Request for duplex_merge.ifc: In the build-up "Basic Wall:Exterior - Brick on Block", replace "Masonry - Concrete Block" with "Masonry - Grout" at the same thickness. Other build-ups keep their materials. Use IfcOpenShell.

First a look at what the model holds.

```python
import ifcopenshell
import ifcopenshell.util.element

model = ifcopenshell.open("duplex_merge.ifc")
print(model.schema)
for layer_set in model.by_type("IfcMaterialLayerSet"):
    if layer_set.LayerSetName == "Basic Wall:Exterior - Brick on Block":
        for layer in layer_set.MaterialLayers:
            print(layer.id(), layer.Material and layer.Material.Name, layer.LayerThickness, sep=" | ")
        print(len(ifcopenshell.util.element.get_elements_by_material(model, layer_set)), "elements and types use it")
print(sorted(m.Name for m in model.by_type("IfcMaterial") if m.Name)[:60])
```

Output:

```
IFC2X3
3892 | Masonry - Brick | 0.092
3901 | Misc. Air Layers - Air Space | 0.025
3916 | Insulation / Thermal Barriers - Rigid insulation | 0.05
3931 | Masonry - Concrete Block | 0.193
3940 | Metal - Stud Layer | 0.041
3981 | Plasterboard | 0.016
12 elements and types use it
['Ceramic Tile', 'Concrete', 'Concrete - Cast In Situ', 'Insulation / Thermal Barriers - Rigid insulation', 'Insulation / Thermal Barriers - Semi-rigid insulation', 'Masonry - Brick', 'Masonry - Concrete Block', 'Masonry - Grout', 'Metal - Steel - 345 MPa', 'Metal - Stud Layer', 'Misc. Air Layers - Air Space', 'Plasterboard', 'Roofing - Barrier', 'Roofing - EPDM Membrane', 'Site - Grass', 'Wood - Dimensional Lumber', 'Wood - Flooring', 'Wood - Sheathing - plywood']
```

```python
import ifcopenshell
import ifcopenshell.api.material

model = ifcopenshell.open("duplex_merge.ifc")

layer_set = next(s for s in model.by_type("IfcMaterialLayerSet") if s.LayerSetName == "Basic Wall:Exterior - Brick on Block")
layer = next(l for l in layer_set.MaterialLayers if l.Material and l.Material.Name == "Masonry - Concrete Block")
material = next(m for m in model.by_type("IfcMaterial") if m.Name == "Masonry - Grout")

# Point this one layer at the other material; renaming the old one would change it everywhere.
ifcopenshell.api.material.edit_layer(model, layer=layer, attributes={}, material=material)

print([l.Material.Name if l.Material else None for l in layer_set.MaterialLayers])

model.write("duplex_merge_edited.ifc")
```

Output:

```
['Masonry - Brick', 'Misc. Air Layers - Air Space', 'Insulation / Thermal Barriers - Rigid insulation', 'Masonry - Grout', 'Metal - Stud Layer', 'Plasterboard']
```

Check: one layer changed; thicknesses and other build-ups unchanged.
